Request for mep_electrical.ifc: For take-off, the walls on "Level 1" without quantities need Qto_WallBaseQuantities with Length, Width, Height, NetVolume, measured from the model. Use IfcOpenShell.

First a look at what the model holds.

```python
import ifcopenshell
import ifcopenshell.util.element
import ifcopenshell.util.unit

model = ifcopenshell.open("mep_electrical.ifc")
print(model.schema)
for unit_type in ("LENGTHUNIT", "AREAUNIT", "VOLUMEUNIT"):
    print(unit_type, ifcopenshell.util.unit.calculate_unit_scale(model, unit_type))
storey = next(s for s in model.by_type("IfcBuildingStorey") if s.Name == "Level 1")
walls = [e for e in ifcopenshell.util.element.get_decomposition(storey) if e.is_a("IfcWall")]
for e in sorted(walls, key=lambda e: e.id()):
    print(e.id(), e.is_a(), e.Name, list(ifcopenshell.util.element.get_psets(e, qtos_only=True)), sep=" | ")
```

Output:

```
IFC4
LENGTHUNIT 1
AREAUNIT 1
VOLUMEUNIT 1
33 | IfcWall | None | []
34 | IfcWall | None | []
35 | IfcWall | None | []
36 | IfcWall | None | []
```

```python
import ifcopenshell
import ifcopenshell.api.pset
import ifcopenshell.geom
import ifcopenshell.util.element
import ifcopenshell.util.shape
import ifcopenshell.util.unit

model = ifcopenshell.open("mep_electrical.ifc")
unit_scale = ifcopenshell.util.unit.calculate_unit_scale(model)
volume_scale = ifcopenshell.util.unit.calculate_unit_scale(model, "VOLUMEUNIT")
settings = ifcopenshell.geom.settings()

storey = next(s for s in model.by_type("IfcBuildingStorey") if s.Name == "Level 1")
walls = [e for e in ifcopenshell.util.element.get_decomposition(storey) if e.is_a("IfcWall")]

for e in sorted(walls, key=lambda e: e.id()):
    if ifcopenshell.util.element.get_psets(e, qtos_only=True, should_inherit=False):
        continue
    # Geometry comes back in metres, in the element's own axes.
    shape = ifcopenshell.geom.create_shape(settings, e)
    values = {
        "Length": ifcopenshell.util.shape.get_x(shape.geometry) / unit_scale,
        "Width": ifcopenshell.util.shape.get_y(shape.geometry) / unit_scale,
        "Height": ifcopenshell.util.shape.get_z(shape.geometry) / unit_scale,
        "NetVolume": ifcopenshell.util.shape.get_volume(shape.geometry) / volume_scale,
    }
    qto = ifcopenshell.api.pset.add_qto(model, product=e, name="Qto_WallBaseQuantities")
    ifcopenshell.api.pset.edit_qto(model, qto=qto, properties=values)
    print(e.id(), {k: round(v, 3) for k, v in values.items()})

model.write("mep_electrical_edited.ifc")
```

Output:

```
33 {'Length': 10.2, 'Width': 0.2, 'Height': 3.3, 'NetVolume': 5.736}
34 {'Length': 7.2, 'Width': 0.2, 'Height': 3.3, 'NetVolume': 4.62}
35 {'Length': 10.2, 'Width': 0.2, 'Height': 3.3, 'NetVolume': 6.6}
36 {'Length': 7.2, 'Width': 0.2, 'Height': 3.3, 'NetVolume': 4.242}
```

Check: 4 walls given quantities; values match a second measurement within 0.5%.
